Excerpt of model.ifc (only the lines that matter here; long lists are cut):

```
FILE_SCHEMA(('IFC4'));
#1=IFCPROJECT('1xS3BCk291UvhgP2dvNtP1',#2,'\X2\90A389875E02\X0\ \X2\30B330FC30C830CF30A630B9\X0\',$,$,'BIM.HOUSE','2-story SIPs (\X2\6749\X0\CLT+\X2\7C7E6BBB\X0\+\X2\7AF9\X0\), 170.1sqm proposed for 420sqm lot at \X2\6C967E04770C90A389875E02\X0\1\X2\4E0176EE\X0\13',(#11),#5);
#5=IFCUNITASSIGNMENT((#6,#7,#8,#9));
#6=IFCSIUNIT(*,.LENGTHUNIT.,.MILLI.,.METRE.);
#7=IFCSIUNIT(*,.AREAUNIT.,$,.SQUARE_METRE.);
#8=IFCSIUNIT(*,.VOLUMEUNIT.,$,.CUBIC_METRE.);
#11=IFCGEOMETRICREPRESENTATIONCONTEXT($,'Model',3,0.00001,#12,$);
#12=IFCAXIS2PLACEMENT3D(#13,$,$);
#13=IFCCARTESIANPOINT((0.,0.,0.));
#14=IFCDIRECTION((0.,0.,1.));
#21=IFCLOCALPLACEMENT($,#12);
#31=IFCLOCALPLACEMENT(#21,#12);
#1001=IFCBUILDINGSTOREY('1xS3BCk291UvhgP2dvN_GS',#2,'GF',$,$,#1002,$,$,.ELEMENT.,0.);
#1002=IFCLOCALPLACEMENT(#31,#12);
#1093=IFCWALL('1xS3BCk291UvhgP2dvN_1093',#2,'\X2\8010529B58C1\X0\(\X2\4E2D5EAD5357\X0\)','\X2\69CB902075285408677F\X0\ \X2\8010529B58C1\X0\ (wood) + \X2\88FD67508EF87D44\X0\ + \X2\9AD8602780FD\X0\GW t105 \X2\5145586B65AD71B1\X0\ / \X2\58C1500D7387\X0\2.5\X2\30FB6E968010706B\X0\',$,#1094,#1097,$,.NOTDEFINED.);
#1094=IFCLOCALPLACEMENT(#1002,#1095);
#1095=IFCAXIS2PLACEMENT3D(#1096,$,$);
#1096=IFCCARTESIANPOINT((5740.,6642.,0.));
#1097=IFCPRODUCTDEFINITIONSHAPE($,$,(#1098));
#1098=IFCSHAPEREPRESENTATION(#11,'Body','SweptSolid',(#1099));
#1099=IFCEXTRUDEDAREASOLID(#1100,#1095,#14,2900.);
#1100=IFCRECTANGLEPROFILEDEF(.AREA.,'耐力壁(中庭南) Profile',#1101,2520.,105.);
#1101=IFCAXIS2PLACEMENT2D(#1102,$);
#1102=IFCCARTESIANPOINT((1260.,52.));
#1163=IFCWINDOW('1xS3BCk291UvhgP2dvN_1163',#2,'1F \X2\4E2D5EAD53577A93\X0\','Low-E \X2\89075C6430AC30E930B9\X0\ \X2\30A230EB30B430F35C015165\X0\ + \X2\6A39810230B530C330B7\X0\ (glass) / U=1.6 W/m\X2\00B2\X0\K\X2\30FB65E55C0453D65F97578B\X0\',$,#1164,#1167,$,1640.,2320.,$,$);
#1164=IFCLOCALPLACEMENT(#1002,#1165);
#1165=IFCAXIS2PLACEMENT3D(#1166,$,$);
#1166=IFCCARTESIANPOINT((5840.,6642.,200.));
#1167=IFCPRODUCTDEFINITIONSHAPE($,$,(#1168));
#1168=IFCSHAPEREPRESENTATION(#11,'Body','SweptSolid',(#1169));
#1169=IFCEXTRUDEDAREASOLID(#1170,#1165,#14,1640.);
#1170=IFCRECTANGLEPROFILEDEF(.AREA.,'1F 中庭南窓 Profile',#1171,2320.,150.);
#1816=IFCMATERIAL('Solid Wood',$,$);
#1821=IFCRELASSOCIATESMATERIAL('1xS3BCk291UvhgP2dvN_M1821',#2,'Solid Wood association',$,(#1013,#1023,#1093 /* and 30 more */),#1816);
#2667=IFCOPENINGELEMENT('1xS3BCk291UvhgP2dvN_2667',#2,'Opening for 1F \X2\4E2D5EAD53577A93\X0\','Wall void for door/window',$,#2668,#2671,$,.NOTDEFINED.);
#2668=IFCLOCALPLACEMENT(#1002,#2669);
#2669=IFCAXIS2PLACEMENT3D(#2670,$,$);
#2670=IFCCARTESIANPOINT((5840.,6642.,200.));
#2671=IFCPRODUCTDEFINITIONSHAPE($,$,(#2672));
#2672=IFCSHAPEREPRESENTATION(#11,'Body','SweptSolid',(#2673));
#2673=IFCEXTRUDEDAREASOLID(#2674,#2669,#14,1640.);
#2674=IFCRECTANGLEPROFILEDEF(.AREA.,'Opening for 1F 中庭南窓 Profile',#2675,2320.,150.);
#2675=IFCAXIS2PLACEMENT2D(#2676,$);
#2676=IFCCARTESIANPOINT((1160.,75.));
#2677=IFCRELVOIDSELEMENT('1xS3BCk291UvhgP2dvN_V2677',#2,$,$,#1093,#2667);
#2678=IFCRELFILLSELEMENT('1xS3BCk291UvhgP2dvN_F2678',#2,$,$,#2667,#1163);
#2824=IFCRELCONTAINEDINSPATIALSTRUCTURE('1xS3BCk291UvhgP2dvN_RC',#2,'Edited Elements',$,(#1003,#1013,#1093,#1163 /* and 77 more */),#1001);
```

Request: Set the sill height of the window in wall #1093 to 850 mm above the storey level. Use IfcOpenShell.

```python
import numpy as np
import ifcopenshell
import ifcopenshell.api.geometry
import ifcopenshell.geom
import ifcopenshell.util.element
import ifcopenshell.util.placement
import ifcopenshell.util.shape
import ifcopenshell.util.unit

model = ifcopenshell.open("model.ifc")
unit_scale = ifcopenshell.util.unit.calculate_unit_scale(model)

window = model.by_id(1163)
opening = window.FillsVoids[0].RelatingOpeningElement
storey = ifcopenshell.util.element.get_container(window, ifc_class="IfcBuildingStorey")
level = ifcopenshell.util.placement.get_local_placement(storey.ObjectPlacement)[2, 3]

# The opening's origin need not be at the sill, so measure its lowest point.
shape = ifcopenshell.geom.create_shape(ifcopenshell.geom.settings(), opening)
bottom = ifcopenshell.util.shape.get_shape_bottom_elevation(shape, shape.geometry) / unit_scale
dz = level + 0.85 / unit_scale - bottom

shift = np.array([0.0, 0.0, dz])
# The window is not placed relative to its opening, so move both.
for product in (opening, window):
    matrix = ifcopenshell.util.placement.get_local_placement(product.ObjectPlacement)
    matrix[:3, 3] += shift
    ifcopenshell.api.geometry.edit_object_placement(model, product=product, matrix=matrix, is_si=False)

print(f"moved by {dz * unit_scale:+.3f} m")

model.write("model-out.ifc")
```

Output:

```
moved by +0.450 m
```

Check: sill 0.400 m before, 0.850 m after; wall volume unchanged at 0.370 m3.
